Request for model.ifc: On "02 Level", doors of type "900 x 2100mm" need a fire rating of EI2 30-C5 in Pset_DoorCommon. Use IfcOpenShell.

First a look at what the model holds.

```python
import ifcopenshell
import ifcopenshell.util.element

model = ifcopenshell.open("model.ifc")
print(model.schema)
storey = next(s for s in model.by_type("IfcBuildingStorey") if s.Name == "02 Level")
doors = [e for e in ifcopenshell.util.element.get_decomposition(storey) if e.is_a("IfcDoor")]
seen = {}
for e in doors:
    element_type = ifcopenshell.util.element.get_type(e)
    key = (element_type.Name if element_type != e and element_type else None, ifcopenshell.util.element.get_pset(e, "Pset_DoorCommon", "FireRating"))
    seen[key] = seen.get(key, 0) + 1
for (name, value), count in sorted(seen.items(), key=str):
    print(count, "x", name, "|", value)
```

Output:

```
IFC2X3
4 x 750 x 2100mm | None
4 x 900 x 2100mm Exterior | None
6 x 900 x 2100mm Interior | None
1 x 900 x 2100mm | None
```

```python
import ifcopenshell
import ifcopenshell.api.pset
import ifcopenshell.util.element

model = ifcopenshell.open("model.ifc")

storey = next(s for s in model.by_type("IfcBuildingStorey") if s.Name == "02 Level")
doors = [e for e in ifcopenshell.util.element.get_decomposition(storey) if e.is_a("IfcDoor")]

count = 0
for e in doors:
    element_type = ifcopenshell.util.element.get_type(e)
    if element_type in (None, e) or element_type.Name != "900 x 2100mm":
        continue
    # add_pset returns the element's existing set when there is one.
    pset = ifcopenshell.api.pset.add_pset(model, product=e, name="Pset_DoorCommon")
    ifcopenshell.api.pset.edit_pset(model, pset=pset, properties={"FireRating": "EI2 30-C5"})
    count += 1

print(count, "doors updated")

model.write("model_rev.ifc")
```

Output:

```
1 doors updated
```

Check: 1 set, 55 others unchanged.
